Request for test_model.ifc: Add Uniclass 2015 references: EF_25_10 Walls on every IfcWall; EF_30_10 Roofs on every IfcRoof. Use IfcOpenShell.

First a look at what the model holds.

```python
import ifcopenshell

model = ifcopenshell.open("test_model.ifc")
print(model.schema)
print("classifications:", [c.Name for c in model.by_type("IfcClassification")])
for ifc_class in ("IfcDoor", "IfcRoof", "IfcStair", "IfcWall", "IfcWindow"):
    print(ifc_class, len(model.by_type(ifc_class)))
```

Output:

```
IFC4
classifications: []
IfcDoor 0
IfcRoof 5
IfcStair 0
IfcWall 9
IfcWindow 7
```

```python
import ifcopenshell
import ifcopenshell.api.classification

model = ifcopenshell.open("test_model.ifc")

system = ifcopenshell.api.classification.add_classification(model, classification="Uniclass 2015")

codes = {
    "IfcWall": ("EF_25_10", "Walls"),
    "IfcRoof": ("EF_30_10", "Roofs"),
}
for ifc_class, (code, name) in codes.items():
    products = model.by_type(ifc_class)
    ifcopenshell.api.classification.add_reference(
        model, products=products, classification=system, identification=code, name=name
    )
    print(code, len(products))

model.write("test_model_edited.ifc")
```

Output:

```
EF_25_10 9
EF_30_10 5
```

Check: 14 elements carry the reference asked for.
